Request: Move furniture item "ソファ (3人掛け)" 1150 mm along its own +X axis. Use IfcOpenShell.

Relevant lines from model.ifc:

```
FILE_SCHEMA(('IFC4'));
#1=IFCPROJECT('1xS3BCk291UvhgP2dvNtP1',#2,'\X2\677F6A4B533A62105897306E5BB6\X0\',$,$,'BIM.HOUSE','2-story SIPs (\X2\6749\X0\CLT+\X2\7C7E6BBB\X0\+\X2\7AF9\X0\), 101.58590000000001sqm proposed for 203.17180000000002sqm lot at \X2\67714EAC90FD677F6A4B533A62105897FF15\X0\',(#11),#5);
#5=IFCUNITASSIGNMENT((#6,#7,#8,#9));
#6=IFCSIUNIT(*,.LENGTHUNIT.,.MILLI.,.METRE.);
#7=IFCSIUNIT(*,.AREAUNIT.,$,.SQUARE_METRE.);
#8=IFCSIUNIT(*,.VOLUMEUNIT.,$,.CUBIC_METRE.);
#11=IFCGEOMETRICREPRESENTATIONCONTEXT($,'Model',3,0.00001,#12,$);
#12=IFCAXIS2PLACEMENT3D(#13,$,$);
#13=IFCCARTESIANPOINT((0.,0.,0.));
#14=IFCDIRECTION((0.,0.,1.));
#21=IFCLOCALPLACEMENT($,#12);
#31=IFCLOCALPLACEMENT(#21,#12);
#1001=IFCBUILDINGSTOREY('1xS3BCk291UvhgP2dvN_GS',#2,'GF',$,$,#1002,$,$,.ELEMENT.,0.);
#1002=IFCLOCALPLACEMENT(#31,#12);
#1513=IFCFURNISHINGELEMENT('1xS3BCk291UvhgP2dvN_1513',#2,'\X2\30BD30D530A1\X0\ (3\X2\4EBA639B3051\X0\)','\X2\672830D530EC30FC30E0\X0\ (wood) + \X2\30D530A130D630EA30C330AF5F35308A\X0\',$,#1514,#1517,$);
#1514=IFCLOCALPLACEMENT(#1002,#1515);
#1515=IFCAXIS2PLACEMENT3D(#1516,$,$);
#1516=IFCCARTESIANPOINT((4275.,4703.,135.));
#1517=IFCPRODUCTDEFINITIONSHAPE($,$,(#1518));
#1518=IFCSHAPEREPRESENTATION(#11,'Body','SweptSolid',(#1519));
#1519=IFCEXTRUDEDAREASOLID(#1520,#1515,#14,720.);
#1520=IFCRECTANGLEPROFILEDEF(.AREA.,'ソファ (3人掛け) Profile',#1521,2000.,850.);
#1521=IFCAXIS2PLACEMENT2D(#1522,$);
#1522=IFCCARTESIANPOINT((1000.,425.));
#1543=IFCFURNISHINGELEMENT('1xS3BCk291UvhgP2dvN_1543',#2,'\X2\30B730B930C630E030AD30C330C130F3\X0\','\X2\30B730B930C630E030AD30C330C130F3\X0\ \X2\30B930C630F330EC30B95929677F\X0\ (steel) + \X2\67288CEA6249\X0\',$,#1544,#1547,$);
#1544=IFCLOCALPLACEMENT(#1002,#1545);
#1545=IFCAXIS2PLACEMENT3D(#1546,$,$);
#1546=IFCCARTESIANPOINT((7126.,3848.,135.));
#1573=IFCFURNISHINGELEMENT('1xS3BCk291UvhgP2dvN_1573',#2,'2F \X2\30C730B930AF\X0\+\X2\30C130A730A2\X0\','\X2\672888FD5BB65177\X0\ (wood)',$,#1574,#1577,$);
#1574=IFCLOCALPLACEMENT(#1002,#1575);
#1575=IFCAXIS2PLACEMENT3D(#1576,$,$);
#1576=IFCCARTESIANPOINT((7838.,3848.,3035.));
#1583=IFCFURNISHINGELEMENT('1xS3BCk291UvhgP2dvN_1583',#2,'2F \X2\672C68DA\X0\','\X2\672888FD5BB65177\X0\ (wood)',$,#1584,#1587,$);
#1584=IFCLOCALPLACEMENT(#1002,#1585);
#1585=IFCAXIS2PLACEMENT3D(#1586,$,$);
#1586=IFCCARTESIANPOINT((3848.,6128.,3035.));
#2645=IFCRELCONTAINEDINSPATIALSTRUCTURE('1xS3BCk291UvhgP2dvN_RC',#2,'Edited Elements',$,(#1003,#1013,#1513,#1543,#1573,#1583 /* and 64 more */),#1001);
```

```python
import ifcopenshell
import ifcopenshell.api.geometry
import ifcopenshell.util.placement

model = ifcopenshell.open("model.ifc")

item = model.by_guid("1xS3BCk291UvhgP2dvN_1513")
matrix = ifcopenshell.util.placement.get_local_placement(item.ObjectPlacement)
matrix[:3, 3] += matrix[:3, 0] * 1150.0
ifcopenshell.api.geometry.edit_object_placement(model, product=item, matrix=matrix, is_si=False)

print(ifcopenshell.util.placement.get_local_placement(item.ObjectPlacement).round(3) + 0.0)

model.write("model_rev.ifc")
```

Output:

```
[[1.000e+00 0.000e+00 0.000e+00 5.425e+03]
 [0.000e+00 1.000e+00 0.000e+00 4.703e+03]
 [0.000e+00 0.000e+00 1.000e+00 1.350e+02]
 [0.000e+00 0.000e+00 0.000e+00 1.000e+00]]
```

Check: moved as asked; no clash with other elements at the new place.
